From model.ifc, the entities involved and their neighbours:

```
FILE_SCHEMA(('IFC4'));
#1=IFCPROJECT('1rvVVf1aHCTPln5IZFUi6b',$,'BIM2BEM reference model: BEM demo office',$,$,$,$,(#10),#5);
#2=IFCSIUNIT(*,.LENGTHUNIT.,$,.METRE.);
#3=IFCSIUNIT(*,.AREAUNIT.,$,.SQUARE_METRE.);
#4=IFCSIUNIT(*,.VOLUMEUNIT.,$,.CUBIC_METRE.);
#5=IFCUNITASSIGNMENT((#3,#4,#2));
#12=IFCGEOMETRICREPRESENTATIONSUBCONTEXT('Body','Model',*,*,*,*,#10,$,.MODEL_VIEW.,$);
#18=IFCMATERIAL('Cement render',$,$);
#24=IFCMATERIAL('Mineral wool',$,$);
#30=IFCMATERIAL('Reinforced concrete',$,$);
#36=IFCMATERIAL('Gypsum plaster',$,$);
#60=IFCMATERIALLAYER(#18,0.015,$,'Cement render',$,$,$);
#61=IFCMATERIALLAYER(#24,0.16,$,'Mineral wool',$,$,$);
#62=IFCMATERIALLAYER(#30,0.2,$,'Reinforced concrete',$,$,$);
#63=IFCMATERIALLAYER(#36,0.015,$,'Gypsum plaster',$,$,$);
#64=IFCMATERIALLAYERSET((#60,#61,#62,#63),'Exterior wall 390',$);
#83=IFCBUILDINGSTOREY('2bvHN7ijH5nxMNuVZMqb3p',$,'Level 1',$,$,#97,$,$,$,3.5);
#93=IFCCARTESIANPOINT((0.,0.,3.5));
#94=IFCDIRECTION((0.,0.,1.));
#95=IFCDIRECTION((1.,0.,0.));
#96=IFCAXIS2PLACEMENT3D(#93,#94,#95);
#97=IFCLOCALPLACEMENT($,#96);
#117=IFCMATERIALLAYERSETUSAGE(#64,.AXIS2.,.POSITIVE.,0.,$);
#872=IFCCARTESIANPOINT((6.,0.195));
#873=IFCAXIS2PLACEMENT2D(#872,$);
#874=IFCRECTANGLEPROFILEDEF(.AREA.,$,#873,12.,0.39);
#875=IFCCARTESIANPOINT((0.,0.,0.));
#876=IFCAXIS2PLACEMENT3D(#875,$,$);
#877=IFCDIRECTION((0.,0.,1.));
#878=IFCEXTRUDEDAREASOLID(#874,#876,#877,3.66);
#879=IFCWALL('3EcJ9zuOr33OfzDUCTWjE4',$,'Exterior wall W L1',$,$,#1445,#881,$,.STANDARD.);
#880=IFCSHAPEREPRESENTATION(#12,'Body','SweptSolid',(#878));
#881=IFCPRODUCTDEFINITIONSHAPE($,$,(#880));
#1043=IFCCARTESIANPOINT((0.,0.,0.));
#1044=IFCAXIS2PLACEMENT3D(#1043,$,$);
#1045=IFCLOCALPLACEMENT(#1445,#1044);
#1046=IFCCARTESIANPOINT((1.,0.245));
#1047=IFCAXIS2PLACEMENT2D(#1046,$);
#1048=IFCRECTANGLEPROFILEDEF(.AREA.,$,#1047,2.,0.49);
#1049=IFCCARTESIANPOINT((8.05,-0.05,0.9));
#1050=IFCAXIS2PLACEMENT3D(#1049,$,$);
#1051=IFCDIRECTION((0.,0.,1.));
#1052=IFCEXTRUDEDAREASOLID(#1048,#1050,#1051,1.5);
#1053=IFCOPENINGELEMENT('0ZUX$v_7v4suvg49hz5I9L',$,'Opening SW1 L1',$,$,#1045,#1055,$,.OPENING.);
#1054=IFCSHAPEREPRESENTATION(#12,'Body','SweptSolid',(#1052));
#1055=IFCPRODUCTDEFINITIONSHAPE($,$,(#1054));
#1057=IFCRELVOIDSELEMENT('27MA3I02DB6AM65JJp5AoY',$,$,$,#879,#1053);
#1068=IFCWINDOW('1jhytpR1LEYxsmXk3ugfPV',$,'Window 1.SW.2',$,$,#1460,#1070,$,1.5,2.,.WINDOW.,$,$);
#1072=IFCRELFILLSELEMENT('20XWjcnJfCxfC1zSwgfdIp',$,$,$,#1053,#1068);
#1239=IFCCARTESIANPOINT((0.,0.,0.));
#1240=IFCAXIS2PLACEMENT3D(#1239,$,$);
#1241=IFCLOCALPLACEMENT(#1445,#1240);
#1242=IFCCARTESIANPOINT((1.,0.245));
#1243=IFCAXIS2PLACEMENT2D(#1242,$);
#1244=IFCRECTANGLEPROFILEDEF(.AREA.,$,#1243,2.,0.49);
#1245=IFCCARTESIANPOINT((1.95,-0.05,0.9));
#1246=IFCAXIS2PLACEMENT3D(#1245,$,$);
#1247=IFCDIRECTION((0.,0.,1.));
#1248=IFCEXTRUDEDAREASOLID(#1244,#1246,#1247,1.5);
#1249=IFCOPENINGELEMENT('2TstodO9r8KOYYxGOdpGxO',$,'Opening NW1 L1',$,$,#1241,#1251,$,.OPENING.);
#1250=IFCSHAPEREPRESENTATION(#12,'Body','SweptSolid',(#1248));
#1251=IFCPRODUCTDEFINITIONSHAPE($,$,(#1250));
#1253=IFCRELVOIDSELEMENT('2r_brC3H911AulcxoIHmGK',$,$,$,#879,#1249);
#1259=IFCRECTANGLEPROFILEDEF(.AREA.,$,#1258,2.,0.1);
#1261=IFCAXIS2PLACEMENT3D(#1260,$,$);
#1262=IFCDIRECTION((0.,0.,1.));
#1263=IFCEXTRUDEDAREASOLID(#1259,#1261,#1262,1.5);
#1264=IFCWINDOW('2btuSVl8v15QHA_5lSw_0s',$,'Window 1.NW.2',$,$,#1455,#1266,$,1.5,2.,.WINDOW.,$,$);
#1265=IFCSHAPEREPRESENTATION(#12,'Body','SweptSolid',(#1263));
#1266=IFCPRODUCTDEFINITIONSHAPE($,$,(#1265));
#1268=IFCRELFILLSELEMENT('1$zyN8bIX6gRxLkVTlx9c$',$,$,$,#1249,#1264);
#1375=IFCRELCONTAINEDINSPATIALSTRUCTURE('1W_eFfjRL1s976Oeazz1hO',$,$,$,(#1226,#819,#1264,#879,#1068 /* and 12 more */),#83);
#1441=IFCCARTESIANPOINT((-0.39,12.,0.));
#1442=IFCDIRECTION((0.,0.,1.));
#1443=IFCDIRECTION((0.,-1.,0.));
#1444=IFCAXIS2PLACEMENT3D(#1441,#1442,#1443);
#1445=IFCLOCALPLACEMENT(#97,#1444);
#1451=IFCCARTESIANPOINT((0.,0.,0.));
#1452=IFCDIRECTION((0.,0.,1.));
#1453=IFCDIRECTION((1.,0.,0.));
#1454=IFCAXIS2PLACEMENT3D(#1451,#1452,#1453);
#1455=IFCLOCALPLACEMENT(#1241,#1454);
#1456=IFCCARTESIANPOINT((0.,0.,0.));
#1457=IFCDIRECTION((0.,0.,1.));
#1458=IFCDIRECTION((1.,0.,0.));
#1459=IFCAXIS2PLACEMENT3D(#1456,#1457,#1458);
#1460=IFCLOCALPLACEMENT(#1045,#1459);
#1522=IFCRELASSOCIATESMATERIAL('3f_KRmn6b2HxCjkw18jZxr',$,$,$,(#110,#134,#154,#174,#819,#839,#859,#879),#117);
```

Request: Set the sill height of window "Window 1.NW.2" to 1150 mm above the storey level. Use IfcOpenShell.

```python
import numpy as np
import ifcopenshell
import ifcopenshell.api.geometry
import ifcopenshell.geom
import ifcopenshell.util.element
import ifcopenshell.util.placement
import ifcopenshell.util.shape
import ifcopenshell.util.unit

model = ifcopenshell.open("model.ifc")
unit_scale = ifcopenshell.util.unit.calculate_unit_scale(model)

window = model.by_guid("2btuSVl8v15QHA_5lSw_0s")
opening = window.FillsVoids[0].RelatingOpeningElement
storey = ifcopenshell.util.element.get_container(window, ifc_class="IfcBuildingStorey")
level = ifcopenshell.util.placement.get_local_placement(storey.ObjectPlacement)[2, 3]

# The opening's origin need not be at the sill, so measure its lowest point.
shape = ifcopenshell.geom.create_shape(ifcopenshell.geom.settings(), opening)
bottom = ifcopenshell.util.shape.get_shape_bottom_elevation(shape, shape.geometry) / unit_scale
dz = level + 1.15 - bottom

shift = np.array([0.0, 0.0, dz])
# The window is placed relative to its opening, so it follows when the opening moves.
matrix = ifcopenshell.util.placement.get_local_placement(opening.ObjectPlacement)
matrix[:3, 3] += shift
ifcopenshell.api.geometry.edit_object_placement(
    model, product=opening, matrix=matrix, is_si=False, should_transform_children=True
)

print(f"moved by {dz * unit_scale:+.3f} m")

model.write("model_rev.ifc")
```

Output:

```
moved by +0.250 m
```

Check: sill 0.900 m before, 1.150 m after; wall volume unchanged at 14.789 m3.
